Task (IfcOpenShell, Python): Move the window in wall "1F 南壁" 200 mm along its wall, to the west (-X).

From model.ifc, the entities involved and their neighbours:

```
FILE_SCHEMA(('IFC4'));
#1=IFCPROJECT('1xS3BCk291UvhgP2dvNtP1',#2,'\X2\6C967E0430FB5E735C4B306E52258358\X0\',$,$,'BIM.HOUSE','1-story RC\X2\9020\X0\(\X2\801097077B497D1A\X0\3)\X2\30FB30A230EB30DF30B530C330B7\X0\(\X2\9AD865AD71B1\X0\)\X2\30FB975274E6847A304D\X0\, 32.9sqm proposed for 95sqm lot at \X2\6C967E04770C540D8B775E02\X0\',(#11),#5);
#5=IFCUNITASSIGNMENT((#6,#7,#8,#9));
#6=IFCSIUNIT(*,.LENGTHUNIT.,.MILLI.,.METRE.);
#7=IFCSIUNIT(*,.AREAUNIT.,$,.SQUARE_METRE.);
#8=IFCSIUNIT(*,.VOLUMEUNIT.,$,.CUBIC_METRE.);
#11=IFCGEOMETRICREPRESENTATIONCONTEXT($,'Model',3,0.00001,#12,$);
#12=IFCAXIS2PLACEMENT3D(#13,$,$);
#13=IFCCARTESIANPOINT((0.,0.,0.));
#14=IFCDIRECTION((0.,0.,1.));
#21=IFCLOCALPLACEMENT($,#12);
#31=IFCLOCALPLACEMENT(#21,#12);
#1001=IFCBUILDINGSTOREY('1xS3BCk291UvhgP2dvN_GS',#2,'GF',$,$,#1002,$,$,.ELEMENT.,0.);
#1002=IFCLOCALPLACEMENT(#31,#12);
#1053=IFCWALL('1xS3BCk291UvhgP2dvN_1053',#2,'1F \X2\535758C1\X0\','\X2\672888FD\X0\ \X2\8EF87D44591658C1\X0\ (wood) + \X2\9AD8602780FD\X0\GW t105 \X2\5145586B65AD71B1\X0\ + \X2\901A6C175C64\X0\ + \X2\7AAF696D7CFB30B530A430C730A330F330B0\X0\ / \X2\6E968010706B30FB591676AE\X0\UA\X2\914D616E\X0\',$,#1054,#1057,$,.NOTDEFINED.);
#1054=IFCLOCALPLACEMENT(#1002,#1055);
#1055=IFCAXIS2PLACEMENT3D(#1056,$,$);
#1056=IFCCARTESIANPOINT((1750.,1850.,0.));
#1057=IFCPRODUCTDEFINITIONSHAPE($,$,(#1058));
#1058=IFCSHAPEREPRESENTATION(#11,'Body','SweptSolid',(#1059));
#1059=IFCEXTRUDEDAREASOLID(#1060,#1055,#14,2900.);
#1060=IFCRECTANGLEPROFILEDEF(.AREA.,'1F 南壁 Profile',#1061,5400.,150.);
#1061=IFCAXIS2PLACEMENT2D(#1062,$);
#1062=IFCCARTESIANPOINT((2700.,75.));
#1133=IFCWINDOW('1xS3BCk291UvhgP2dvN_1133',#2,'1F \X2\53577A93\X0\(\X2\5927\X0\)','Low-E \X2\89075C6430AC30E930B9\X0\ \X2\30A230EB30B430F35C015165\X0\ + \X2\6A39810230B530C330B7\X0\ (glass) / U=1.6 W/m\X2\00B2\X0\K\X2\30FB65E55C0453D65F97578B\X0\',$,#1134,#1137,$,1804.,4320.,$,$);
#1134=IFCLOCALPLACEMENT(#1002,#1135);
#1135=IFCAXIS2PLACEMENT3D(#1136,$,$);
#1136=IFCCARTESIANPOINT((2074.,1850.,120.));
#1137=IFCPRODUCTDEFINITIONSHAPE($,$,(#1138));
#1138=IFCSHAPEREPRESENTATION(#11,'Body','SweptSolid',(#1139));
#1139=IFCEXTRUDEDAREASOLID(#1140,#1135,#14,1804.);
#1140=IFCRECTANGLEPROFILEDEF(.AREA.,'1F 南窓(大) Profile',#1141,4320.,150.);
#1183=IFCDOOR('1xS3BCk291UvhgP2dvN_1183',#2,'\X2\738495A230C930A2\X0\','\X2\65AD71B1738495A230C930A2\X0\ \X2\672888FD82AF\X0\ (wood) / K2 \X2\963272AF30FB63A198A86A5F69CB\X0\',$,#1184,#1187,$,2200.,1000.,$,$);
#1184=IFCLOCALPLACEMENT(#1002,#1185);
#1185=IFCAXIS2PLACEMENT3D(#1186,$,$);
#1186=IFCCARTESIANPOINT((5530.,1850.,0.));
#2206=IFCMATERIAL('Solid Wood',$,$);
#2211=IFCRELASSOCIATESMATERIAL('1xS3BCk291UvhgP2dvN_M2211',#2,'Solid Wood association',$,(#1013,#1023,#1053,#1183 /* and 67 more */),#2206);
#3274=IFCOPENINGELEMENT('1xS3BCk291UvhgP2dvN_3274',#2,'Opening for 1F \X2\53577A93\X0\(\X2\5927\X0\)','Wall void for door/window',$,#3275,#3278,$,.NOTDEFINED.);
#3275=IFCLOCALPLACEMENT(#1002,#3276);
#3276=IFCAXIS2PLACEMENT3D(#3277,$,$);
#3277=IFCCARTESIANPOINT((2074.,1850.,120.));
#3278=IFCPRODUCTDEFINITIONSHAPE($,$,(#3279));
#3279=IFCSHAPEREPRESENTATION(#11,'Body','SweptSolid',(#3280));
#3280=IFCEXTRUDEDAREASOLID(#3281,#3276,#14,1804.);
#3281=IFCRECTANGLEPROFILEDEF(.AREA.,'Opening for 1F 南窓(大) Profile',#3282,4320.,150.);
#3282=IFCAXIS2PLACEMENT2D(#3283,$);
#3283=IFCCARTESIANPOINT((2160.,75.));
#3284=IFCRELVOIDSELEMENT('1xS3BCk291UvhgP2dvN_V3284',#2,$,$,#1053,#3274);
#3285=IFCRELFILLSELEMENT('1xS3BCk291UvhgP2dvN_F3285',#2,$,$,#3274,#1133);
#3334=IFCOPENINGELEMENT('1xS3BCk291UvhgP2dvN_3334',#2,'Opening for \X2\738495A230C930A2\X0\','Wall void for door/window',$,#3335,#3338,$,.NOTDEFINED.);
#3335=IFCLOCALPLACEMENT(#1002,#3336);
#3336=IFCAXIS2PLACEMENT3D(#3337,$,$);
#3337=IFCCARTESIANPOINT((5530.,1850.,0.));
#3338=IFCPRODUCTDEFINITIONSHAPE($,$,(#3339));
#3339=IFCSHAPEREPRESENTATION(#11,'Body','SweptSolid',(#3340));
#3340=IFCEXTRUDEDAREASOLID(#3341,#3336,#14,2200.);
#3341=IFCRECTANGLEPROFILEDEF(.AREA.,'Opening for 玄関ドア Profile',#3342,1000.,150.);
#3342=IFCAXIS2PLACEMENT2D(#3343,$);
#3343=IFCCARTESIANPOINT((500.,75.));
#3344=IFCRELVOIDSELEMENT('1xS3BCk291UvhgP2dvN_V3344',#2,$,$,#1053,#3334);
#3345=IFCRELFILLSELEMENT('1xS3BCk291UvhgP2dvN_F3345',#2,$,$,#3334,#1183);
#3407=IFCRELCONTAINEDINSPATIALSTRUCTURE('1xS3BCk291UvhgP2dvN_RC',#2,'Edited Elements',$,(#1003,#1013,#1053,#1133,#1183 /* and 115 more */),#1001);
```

```python
import ifcopenshell
import ifcopenshell.api.geometry
import ifcopenshell.util.placement
import ifcopenshell.util.unit

model = ifcopenshell.open("model.ifc")
unit_scale = ifcopenshell.util.unit.calculate_unit_scale(model)

window = model.by_id(1133)
opening = window.FillsVoids[0].RelatingOpeningElement
wall = opening.VoidsElements[0].RelatingBuildingElement

wall_matrix = ifcopenshell.util.placement.get_local_placement(wall.ObjectPlacement)
shift = wall_matrix[:3, 0] * -0.2 / unit_scale
before = ifcopenshell.util.placement.get_local_placement(window.ObjectPlacement)[:3, 3].copy()

# The window is not placed relative to its opening, so move both.
for product in (opening, window):
    matrix = ifcopenshell.util.placement.get_local_placement(product.ObjectPlacement)
    matrix[:3, 3] += shift
    ifcopenshell.api.geometry.edit_object_placement(model, product=product, matrix=matrix, is_si=False)

after = ifcopenshell.util.placement.get_local_placement(window.ObjectPlacement)[:3, 3]
print("window moved by", (after - before).round(3) + 0.0)

model.write("model_edited.ifc")
```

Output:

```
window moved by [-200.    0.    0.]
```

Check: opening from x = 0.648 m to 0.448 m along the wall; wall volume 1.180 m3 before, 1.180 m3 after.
